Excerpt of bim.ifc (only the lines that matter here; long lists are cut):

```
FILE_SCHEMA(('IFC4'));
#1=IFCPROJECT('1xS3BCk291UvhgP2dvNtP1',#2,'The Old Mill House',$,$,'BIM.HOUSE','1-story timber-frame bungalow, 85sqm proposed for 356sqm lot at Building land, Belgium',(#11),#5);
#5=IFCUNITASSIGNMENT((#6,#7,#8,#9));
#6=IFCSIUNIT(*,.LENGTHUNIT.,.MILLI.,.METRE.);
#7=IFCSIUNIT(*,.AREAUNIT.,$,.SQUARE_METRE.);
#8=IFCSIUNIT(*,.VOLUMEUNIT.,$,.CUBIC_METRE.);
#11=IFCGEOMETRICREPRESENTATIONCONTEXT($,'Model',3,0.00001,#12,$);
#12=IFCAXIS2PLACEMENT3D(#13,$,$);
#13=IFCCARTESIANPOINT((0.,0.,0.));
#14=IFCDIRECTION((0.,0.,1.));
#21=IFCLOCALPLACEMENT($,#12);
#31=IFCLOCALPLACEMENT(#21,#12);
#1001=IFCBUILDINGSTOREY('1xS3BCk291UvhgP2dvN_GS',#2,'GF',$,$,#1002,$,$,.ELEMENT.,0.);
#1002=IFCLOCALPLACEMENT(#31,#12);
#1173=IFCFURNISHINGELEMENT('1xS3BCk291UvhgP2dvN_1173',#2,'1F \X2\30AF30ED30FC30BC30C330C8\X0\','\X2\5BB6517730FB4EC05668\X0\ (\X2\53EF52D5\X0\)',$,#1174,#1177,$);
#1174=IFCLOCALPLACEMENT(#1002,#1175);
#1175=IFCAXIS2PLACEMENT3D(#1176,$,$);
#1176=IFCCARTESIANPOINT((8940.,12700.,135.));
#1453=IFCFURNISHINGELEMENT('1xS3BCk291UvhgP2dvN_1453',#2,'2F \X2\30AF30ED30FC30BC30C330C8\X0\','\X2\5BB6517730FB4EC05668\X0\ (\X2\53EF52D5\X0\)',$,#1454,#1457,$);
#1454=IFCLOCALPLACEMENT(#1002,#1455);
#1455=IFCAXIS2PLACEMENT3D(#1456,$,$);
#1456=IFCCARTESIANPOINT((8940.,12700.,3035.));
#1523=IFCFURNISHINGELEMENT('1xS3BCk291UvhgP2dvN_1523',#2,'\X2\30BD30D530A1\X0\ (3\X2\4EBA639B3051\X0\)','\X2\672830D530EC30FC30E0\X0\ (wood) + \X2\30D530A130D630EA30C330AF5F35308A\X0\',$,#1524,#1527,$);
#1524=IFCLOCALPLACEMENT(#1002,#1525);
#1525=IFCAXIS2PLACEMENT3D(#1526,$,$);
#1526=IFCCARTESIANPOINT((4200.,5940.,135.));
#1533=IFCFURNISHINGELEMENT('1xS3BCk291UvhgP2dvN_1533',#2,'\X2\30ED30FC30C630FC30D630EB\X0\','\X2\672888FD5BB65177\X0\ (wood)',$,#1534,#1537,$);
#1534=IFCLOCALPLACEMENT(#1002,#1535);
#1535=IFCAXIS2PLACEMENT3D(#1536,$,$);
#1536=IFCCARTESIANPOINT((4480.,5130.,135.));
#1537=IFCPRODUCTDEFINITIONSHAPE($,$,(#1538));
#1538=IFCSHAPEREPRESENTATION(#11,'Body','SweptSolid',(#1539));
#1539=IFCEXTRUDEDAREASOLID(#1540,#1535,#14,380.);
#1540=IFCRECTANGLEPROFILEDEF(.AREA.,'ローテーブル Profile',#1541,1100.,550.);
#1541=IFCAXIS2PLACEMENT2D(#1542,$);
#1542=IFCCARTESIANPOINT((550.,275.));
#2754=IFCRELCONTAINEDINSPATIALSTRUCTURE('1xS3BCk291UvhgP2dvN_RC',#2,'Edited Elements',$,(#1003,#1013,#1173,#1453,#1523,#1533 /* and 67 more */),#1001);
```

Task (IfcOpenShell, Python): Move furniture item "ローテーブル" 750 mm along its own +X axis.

```python
import ifcopenshell
import ifcopenshell.api.geometry
import ifcopenshell.util.placement
import ifcopenshell.util.unit

model = ifcopenshell.open("bim.ifc")
unit_scale = ifcopenshell.util.unit.calculate_unit_scale(model)

item = model.by_id(1533)
matrix = ifcopenshell.util.placement.get_local_placement(item.ObjectPlacement)
matrix[:3, 3] += matrix[:3, 0] * 0.75 / unit_scale
ifcopenshell.api.geometry.edit_object_placement(model, product=item, matrix=matrix, is_si=False)

print(ifcopenshell.util.placement.get_local_placement(item.ObjectPlacement).round(3) + 0.0)

model.write("bim_v2.ifc")
```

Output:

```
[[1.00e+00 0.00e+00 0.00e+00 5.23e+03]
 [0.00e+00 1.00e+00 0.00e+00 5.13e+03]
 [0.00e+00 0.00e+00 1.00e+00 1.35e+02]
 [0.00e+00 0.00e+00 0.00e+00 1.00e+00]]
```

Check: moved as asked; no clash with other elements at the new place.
